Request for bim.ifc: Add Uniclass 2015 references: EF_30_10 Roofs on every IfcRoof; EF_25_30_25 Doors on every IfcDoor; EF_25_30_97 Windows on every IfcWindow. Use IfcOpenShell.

First a look at what the model holds.

```python
import ifcopenshell

model = ifcopenshell.open("bim.ifc")
print(model.schema)
print("classifications:", [c.Name for c in model.by_type("IfcClassification")])
for ifc_class in ("IfcDoor", "IfcRoof", "IfcStair", "IfcWall", "IfcWindow"):
    print(ifc_class, len(model.by_type(ifc_class)))
```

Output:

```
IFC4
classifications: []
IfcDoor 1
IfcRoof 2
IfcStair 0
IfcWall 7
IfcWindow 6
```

```python
import ifcopenshell
import ifcopenshell.api.classification

model = ifcopenshell.open("bim.ifc")

system = ifcopenshell.api.classification.add_classification(model, classification="Uniclass 2015")

codes = {
    "IfcRoof": ("EF_30_10", "Roofs"),
    "IfcDoor": ("EF_25_30_25", "Doors"),
    "IfcWindow": ("EF_25_30_97", "Windows"),
}
for ifc_class, (code, name) in codes.items():
    products = model.by_type(ifc_class)
    ifcopenshell.api.classification.add_reference(
        model, products=products, classification=system, identification=code, name=name
    )
    print(code, len(products))

model.write("bim-out.ifc")
```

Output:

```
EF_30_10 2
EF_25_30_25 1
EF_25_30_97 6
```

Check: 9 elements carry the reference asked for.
